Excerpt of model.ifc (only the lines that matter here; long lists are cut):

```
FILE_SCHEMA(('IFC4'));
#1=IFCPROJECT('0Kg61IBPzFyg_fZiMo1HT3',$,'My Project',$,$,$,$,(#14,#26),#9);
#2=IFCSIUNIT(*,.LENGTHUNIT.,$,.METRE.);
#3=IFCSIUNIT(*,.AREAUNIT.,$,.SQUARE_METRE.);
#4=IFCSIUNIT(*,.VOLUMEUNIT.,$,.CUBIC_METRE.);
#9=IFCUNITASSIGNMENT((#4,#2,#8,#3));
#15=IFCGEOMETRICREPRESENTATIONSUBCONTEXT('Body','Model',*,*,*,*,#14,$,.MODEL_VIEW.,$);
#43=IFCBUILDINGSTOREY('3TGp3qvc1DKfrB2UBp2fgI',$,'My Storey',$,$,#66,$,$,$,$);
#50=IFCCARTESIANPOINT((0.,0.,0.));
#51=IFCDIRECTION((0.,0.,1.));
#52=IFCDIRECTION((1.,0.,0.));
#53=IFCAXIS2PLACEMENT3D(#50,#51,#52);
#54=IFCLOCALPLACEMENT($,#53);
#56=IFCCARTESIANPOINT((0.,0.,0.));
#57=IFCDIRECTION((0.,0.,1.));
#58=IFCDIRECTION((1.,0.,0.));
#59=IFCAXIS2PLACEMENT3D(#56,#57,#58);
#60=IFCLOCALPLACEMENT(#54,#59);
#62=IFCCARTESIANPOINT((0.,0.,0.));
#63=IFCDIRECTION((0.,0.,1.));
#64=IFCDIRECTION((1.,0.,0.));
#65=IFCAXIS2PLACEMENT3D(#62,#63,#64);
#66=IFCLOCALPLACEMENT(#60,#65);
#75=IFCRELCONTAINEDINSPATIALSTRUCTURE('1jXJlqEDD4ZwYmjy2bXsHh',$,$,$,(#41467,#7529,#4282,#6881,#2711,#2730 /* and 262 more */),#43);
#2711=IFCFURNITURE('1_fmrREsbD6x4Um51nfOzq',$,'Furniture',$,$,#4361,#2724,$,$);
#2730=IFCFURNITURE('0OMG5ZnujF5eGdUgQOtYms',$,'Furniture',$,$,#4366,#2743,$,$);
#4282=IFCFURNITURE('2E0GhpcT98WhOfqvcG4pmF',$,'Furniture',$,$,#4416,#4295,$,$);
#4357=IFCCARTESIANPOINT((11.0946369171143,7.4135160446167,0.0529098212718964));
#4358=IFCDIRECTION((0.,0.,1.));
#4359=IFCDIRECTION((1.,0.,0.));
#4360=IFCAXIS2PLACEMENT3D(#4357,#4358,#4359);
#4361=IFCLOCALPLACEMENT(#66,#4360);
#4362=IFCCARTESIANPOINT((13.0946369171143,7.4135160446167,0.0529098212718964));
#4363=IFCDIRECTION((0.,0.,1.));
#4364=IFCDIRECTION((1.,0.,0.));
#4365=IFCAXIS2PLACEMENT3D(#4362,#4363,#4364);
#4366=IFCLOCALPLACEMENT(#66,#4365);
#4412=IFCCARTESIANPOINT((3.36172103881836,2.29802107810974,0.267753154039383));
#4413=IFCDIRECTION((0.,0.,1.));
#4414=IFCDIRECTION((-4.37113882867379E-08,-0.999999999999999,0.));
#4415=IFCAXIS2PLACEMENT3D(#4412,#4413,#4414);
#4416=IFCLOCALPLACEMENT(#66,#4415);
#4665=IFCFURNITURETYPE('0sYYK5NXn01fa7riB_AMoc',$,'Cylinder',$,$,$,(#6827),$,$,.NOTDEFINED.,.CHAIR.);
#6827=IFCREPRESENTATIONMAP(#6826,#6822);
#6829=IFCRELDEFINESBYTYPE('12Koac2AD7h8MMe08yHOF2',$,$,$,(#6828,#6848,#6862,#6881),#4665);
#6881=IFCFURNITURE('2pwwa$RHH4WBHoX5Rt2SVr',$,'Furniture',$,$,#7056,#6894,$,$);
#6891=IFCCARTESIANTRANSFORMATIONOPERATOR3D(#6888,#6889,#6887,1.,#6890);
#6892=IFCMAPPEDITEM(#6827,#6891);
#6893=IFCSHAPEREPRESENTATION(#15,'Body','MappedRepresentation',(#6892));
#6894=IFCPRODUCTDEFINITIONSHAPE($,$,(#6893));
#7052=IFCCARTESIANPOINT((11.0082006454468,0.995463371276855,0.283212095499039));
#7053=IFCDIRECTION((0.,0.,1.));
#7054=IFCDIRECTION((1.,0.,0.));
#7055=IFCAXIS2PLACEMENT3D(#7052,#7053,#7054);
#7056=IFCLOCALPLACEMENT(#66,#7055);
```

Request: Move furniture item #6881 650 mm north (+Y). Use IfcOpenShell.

```python
import ifcopenshell
import ifcopenshell.api.geometry
import ifcopenshell.util.placement

model = ifcopenshell.open("model.ifc")

item = model.by_id(6881)
matrix = ifcopenshell.util.placement.get_local_placement(item.ObjectPlacement)
matrix[1, 3] += 0.65
ifcopenshell.api.geometry.edit_object_placement(model, product=item, matrix=matrix, is_si=False)

print(ifcopenshell.util.placement.get_local_placement(item.ObjectPlacement).round(3) + 0.0)

model.write("model_v2.ifc")
```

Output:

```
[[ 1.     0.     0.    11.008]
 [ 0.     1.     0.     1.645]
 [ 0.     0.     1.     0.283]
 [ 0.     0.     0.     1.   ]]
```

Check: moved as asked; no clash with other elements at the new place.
